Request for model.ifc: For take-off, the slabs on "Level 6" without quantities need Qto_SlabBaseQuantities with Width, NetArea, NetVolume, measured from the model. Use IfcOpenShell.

First a look at what the model holds.

```python
import ifcopenshell
import ifcopenshell.util.element
import ifcopenshell.util.unit

model = ifcopenshell.open("model.ifc")
print(model.schema)
for unit_type in ("LENGTHUNIT", "AREAUNIT", "VOLUMEUNIT"):
    print(unit_type, ifcopenshell.util.unit.calculate_unit_scale(model, unit_type))
storey = next(s for s in model.by_type("IfcBuildingStorey") if s.Name == "Level 6")
slabs = [e for e in ifcopenshell.util.element.get_decomposition(storey) if e.is_a("IfcSlab")]
for e in sorted(slabs, key=lambda e: e.id()):
    print(e.id(), e.is_a(), e.Name, list(ifcopenshell.util.element.get_psets(e, qtos_only=True)), sep=" | ")
```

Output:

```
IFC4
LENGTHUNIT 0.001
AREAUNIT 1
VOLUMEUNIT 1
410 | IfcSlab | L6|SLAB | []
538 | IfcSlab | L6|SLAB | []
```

```python
import ifcopenshell
import ifcopenshell.api.pset
import ifcopenshell.geom
import ifcopenshell.util.element
import ifcopenshell.util.shape
import ifcopenshell.util.unit

model = ifcopenshell.open("model.ifc")
unit_scale = ifcopenshell.util.unit.calculate_unit_scale(model)
area_scale = ifcopenshell.util.unit.calculate_unit_scale(model, "AREAUNIT")
volume_scale = ifcopenshell.util.unit.calculate_unit_scale(model, "VOLUMEUNIT")
settings = ifcopenshell.geom.settings()

storey = next(s for s in model.by_type("IfcBuildingStorey") if s.Name == "Level 6")
slabs = [e for e in ifcopenshell.util.element.get_decomposition(storey) if e.is_a("IfcSlab")]

for e in sorted(slabs, key=lambda e: e.id()):
    if ifcopenshell.util.element.get_psets(e, qtos_only=True, should_inherit=False):
        continue
    # Geometry comes back in metres, in the element's own axes.
    shape = ifcopenshell.geom.create_shape(settings, e)
    values = {
        "Width": ifcopenshell.util.shape.get_z(shape.geometry) / unit_scale,
        "NetArea": ifcopenshell.util.shape.get_footprint_area(shape.geometry) / area_scale,
        "NetVolume": ifcopenshell.util.shape.get_volume(shape.geometry) / volume_scale,
    }
    qto = ifcopenshell.api.pset.add_qto(model, product=e, name="Qto_SlabBaseQuantities")
    ifcopenshell.api.pset.edit_qto(model, qto=qto, properties=values)
    print(e.id(), {k: round(v, 3) for k, v in values.items()})

model.write("model_updated.ifc")
```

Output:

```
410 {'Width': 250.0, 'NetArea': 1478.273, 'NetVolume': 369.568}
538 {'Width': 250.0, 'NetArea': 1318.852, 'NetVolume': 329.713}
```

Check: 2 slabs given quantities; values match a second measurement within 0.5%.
